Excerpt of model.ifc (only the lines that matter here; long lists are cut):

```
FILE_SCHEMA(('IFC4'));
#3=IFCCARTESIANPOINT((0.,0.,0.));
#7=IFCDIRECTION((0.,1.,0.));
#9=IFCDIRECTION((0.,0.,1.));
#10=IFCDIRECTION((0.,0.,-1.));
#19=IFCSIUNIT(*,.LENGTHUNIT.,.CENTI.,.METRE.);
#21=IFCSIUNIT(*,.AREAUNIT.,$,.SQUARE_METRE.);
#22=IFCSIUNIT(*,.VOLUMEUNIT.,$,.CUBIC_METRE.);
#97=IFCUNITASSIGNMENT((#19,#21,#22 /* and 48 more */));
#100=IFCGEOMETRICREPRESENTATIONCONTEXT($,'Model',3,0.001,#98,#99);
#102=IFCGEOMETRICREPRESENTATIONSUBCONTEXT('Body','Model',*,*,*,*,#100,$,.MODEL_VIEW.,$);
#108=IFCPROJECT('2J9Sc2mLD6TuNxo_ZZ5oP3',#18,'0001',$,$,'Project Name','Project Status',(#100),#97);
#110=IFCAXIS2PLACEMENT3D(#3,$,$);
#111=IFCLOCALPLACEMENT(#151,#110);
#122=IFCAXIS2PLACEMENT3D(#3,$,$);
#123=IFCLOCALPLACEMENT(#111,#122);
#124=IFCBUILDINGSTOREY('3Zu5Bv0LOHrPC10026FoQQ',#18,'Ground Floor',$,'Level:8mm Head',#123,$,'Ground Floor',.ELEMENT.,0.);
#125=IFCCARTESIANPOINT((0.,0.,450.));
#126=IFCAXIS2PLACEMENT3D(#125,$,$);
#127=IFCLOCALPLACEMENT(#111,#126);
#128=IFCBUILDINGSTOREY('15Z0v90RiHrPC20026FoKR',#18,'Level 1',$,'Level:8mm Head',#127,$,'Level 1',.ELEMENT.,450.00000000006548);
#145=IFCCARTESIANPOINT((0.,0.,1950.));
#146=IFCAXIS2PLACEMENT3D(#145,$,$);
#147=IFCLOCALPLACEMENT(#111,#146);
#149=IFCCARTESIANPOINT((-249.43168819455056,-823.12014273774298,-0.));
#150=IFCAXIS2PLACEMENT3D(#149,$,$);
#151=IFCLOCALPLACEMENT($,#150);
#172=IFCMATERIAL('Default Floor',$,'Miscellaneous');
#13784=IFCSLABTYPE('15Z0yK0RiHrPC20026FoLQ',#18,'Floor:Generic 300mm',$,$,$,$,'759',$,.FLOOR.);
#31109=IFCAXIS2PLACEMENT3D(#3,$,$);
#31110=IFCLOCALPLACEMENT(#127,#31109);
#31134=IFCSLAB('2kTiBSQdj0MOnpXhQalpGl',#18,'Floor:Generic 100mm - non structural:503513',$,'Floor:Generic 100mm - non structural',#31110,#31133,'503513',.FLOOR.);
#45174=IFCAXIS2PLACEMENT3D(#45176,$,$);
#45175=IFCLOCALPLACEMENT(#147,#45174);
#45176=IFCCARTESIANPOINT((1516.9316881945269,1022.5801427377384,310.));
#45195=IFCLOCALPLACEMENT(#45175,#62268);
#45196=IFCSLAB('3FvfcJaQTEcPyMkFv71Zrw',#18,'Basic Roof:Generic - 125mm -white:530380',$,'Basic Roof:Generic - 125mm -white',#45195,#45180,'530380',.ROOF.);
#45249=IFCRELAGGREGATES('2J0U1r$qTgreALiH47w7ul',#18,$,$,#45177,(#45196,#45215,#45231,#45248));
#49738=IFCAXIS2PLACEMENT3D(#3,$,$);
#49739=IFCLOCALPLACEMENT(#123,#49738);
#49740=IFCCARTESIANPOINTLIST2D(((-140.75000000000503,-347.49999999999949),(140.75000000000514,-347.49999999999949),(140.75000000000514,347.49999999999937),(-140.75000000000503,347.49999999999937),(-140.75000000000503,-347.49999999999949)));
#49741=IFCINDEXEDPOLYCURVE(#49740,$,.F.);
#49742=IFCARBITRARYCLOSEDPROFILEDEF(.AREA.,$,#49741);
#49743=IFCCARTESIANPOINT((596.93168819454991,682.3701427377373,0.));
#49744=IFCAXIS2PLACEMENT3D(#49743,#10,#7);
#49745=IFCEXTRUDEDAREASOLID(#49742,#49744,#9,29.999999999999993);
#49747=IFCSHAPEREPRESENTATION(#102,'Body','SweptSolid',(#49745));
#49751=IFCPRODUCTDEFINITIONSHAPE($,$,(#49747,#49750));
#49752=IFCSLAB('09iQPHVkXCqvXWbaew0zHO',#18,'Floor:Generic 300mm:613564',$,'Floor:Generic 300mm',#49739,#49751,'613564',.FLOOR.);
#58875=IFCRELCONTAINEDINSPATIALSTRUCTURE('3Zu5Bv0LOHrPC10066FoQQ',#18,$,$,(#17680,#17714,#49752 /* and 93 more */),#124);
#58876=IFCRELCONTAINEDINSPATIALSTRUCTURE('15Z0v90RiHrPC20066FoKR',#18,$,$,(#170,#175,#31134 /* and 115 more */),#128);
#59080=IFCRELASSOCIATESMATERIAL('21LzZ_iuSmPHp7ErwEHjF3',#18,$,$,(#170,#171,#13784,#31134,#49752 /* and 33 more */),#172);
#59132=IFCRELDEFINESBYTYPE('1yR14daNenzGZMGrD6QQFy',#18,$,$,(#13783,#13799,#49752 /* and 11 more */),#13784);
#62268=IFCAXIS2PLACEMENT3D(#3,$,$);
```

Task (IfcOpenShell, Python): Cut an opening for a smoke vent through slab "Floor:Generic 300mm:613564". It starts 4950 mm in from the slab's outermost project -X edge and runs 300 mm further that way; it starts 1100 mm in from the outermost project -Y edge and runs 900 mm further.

```python
import numpy as np
import ifcopenshell
import ifcopenshell.api.feature
import ifcopenshell.api.geometry
import ifcopenshell.api.root
import ifcopenshell.geom
import ifcopenshell.util.placement
import ifcopenshell.util.representation
import ifcopenshell.util.shape
import ifcopenshell.util.unit

model = ifcopenshell.open("model.ifc")
unit_scale = ifcopenshell.util.unit.calculate_unit_scale(model)
settings = ifcopenshell.geom.settings()


def volume(element):
    """Net volume in cubic metres, openings subtracted."""
    shape = ifcopenshell.geom.create_shape(settings, element)
    return ifcopenshell.util.shape.get_volume(shape.geometry)


slab = model.by_guid("09iQPHVkXCqvXWbaew0zHO")
before = volume(slab)

# Extent in the slab's own axes, in metres. The edges named are its -X and -Y sides.
slab_shape = ifcopenshell.geom.create_shape(settings, slab)
vertices = ifcopenshell.util.shape.get_vertices(slab_shape.geometry)
x_min, y_min, bottom = vertices.min(axis=0)
top = vertices[:, 2].max()

opening = ifcopenshell.api.root.create_entity(model, ifc_class="IfcOpeningElement", name="Smoke vent opening", predefined_type="OPENING")
context = ifcopenshell.util.representation.get_context(model, "Model", "Body", "MODEL_VIEW")
width, depth = 0.3, 0.9
outline = [(0.0, 0.0), (width, 0.0), (width, depth), (0.0, depth), (0.0, 0.0)]
# Overshoot both faces by 50 mm so the cut is clean.
shape = ifcopenshell.api.geometry.add_slab_representation(
    model, context=context, depth=top - bottom + 0.1, polyline=outline
)
ifcopenshell.api.geometry.assign_representation(model, product=opening, representation=shape)

matrix = ifcopenshell.util.placement.get_local_placement(slab.ObjectPlacement)
matrix[:, 3] = matrix @ np.append(np.array([x_min + 4.95, y_min + 1.1, bottom - 0.05]) / unit_scale, 1.0)
ifcopenshell.api.geometry.edit_object_placement(model, product=opening, matrix=matrix, is_si=False)
ifcopenshell.api.feature.add_feature(model, feature=opening, element=slab)

after = volume(slab)

print(f"slab volume {before:.3f} -> {after:.3f} m3")

model.write("model_v2.ifc")
```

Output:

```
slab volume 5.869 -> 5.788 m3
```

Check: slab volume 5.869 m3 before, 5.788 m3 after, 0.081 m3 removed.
